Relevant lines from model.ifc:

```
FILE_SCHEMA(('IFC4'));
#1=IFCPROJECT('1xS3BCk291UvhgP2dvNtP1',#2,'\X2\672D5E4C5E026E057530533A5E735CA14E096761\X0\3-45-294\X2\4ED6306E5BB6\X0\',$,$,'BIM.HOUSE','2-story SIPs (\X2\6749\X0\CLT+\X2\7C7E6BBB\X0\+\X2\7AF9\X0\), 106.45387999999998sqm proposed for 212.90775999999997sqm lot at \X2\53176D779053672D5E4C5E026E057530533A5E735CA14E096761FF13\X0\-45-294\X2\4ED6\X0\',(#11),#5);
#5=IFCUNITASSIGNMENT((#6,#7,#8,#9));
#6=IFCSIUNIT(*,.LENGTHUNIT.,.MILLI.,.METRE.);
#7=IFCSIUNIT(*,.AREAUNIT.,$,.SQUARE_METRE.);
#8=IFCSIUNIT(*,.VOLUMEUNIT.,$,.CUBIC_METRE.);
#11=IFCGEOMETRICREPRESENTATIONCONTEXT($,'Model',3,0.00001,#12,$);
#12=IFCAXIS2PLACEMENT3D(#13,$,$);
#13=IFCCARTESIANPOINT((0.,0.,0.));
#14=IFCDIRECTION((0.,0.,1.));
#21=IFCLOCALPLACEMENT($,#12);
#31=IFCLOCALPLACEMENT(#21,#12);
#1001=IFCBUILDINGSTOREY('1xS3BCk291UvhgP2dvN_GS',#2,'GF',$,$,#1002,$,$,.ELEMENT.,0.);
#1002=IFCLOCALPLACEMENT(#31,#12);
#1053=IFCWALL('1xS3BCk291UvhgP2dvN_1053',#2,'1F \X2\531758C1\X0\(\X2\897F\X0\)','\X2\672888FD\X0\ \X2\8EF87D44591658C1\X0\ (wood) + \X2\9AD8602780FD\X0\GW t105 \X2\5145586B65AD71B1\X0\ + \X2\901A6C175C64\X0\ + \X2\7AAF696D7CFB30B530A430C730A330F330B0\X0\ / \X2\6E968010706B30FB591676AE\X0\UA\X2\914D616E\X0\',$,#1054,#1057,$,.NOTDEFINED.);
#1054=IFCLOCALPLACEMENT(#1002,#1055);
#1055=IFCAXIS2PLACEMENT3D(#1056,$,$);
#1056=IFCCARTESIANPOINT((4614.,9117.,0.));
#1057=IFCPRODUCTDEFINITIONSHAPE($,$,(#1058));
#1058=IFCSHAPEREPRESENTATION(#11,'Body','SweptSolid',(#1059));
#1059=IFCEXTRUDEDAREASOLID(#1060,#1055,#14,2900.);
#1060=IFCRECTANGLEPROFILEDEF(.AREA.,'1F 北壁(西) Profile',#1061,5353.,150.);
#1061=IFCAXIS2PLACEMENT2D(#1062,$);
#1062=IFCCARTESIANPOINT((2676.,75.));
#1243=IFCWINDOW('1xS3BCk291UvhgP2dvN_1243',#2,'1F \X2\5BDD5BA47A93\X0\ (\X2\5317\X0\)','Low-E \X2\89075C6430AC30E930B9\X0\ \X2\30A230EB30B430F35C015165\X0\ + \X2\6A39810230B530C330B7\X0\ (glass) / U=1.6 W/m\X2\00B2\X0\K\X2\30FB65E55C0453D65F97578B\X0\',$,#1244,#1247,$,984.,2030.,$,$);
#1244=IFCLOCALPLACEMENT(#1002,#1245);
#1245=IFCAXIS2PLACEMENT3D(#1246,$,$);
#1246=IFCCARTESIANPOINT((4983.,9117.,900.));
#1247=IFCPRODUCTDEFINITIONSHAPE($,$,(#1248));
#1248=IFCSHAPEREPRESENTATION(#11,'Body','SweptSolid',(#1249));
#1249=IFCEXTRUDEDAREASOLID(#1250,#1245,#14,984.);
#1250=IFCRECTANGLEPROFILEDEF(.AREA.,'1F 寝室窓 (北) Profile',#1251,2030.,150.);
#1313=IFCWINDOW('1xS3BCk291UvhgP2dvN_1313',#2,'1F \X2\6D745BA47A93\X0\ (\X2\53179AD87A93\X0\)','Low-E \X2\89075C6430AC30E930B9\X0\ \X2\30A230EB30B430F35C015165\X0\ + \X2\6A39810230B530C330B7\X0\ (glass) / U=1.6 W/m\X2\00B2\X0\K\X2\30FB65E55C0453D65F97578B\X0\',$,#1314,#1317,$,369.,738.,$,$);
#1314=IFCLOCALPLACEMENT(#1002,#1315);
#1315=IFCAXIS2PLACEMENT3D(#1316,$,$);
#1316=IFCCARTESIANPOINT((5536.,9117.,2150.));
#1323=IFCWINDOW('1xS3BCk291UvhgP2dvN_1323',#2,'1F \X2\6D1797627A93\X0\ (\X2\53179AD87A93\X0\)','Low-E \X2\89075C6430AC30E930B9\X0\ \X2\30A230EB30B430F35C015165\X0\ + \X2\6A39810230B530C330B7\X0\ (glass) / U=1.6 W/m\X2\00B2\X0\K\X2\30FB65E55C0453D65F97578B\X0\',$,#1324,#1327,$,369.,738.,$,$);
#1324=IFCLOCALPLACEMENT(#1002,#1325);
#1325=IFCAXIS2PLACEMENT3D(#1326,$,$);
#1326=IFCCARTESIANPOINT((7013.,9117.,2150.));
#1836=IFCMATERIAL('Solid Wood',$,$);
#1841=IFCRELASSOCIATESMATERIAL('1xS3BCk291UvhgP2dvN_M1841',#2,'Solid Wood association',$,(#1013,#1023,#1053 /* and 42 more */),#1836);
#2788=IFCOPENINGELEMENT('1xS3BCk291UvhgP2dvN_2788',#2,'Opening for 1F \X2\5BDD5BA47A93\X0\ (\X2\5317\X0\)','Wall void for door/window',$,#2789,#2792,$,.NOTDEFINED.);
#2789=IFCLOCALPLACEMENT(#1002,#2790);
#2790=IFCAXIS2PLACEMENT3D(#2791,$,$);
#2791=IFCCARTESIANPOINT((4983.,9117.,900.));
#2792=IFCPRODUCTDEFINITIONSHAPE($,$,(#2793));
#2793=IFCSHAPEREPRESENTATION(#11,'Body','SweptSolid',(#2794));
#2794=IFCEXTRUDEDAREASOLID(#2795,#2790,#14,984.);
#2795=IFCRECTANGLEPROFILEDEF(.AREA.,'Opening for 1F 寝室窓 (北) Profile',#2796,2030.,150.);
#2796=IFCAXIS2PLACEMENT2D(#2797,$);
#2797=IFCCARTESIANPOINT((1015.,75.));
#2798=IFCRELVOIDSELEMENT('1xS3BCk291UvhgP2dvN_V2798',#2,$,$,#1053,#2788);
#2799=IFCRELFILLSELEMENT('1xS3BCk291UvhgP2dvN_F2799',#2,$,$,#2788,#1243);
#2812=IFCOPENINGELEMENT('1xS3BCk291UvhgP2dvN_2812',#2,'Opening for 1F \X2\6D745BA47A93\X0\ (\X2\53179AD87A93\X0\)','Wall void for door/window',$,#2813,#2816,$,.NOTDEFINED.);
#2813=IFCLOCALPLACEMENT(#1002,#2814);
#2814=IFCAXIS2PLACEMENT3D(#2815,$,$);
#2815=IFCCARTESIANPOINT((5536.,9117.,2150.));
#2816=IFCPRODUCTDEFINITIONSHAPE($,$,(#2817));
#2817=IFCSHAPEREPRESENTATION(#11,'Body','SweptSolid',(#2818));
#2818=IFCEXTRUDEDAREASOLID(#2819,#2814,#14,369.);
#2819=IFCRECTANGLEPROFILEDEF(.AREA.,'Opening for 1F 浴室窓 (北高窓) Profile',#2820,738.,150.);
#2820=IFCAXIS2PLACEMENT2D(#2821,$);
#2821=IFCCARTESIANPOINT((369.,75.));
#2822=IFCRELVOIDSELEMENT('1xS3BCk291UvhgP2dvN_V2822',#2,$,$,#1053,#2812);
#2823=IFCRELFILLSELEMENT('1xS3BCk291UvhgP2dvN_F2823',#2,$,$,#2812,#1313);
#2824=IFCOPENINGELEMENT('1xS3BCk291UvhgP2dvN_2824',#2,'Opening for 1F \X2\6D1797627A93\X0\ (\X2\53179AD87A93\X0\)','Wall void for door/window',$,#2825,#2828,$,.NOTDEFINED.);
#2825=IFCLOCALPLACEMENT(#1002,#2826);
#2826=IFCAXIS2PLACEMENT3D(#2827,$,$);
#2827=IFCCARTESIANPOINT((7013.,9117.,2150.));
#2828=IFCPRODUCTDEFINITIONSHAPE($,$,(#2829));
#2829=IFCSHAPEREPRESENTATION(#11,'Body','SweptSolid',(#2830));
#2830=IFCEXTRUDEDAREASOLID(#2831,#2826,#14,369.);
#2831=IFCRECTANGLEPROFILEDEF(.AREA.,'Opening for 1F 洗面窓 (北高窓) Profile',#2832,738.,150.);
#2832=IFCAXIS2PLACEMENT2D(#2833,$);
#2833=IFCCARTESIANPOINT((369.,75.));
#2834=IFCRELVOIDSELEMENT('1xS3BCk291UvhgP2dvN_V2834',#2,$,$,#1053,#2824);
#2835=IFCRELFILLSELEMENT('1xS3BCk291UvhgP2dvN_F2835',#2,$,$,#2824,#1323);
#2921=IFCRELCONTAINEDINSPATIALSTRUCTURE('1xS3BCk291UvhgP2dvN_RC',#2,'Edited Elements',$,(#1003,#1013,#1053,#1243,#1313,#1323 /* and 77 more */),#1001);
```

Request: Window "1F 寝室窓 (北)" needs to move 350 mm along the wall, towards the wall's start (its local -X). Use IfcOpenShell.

```python
import ifcopenshell
import ifcopenshell.api.geometry
import ifcopenshell.util.placement

model = ifcopenshell.open("model.ifc")

window = model.by_guid("1xS3BCk291UvhgP2dvN_1243")
opening = window.FillsVoids[0].RelatingOpeningElement
wall = opening.VoidsElements[0].RelatingBuildingElement

wall_matrix = ifcopenshell.util.placement.get_local_placement(wall.ObjectPlacement)
shift = wall_matrix[:3, 0] * -350.0
before = ifcopenshell.util.placement.get_local_placement(window.ObjectPlacement)[:3, 3].copy()

# The window is not placed relative to its opening, so move both.
for product in (opening, window):
    matrix = ifcopenshell.util.placement.get_local_placement(product.ObjectPlacement)
    matrix[:3, 3] += shift
    ifcopenshell.api.geometry.edit_object_placement(model, product=product, matrix=matrix, is_si=False)

after = ifcopenshell.util.placement.get_local_placement(window.ObjectPlacement)[:3, 3]
print("window moved by", (after - before).round(3) + 0.0)

model.write("model_updated.ifc")
```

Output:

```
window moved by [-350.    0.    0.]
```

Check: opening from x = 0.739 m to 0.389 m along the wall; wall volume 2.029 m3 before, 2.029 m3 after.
